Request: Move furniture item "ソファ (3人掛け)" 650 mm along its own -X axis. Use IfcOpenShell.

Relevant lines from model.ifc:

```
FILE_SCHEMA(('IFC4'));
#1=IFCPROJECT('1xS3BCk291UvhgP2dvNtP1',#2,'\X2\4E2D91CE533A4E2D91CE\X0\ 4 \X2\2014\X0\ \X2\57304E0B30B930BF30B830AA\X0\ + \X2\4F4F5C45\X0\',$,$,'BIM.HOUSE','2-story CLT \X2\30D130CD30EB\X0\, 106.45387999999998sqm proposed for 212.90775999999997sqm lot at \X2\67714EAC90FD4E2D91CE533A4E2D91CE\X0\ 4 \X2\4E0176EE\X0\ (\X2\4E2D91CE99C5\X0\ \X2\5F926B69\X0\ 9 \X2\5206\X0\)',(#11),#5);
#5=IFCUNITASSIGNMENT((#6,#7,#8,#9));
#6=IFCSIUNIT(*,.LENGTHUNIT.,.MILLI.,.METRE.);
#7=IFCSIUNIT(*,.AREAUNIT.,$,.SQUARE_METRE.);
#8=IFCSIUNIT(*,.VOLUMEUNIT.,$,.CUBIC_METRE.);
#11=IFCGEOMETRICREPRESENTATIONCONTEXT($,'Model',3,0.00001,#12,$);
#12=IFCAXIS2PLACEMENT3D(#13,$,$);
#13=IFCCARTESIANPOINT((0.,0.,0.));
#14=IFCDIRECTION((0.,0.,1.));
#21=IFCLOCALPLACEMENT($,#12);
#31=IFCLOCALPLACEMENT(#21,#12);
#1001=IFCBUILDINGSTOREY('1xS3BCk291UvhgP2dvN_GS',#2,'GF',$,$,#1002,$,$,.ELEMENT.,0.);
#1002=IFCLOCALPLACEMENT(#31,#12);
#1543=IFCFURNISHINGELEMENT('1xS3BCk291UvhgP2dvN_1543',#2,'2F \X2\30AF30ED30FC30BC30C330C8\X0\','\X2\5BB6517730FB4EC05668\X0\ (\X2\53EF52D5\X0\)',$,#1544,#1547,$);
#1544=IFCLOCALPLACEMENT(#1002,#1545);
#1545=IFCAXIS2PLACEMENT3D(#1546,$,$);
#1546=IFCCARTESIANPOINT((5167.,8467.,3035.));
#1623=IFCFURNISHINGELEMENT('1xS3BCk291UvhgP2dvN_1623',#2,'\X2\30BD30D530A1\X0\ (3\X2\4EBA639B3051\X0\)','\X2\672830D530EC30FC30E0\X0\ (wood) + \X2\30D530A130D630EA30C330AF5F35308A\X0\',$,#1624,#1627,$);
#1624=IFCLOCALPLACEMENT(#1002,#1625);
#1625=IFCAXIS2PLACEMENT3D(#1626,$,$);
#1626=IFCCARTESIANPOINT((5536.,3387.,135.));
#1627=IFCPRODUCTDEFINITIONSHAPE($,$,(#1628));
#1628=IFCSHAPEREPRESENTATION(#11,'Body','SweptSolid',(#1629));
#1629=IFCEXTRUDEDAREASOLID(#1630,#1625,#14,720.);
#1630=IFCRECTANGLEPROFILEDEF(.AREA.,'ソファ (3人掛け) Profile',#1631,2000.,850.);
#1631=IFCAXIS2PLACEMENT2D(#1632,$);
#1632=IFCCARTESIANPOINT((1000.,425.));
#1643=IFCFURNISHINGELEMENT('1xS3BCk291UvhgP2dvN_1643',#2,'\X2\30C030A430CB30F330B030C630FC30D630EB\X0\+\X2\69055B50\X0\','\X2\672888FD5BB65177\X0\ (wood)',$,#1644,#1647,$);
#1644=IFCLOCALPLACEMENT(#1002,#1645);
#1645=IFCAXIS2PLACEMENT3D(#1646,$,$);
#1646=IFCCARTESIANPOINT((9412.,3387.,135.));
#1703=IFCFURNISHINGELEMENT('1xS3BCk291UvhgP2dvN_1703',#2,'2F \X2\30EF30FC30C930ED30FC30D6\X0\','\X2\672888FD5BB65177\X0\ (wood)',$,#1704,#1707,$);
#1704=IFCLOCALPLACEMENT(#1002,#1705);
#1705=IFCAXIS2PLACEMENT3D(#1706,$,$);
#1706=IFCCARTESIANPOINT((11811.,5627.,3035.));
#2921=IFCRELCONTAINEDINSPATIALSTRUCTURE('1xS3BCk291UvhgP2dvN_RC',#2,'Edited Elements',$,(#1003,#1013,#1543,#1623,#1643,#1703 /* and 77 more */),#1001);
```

```python
import ifcopenshell
import ifcopenshell.api.geometry
import ifcopenshell.util.placement

model = ifcopenshell.open("model.ifc")

item = model.by_id(1623)
matrix = ifcopenshell.util.placement.get_local_placement(item.ObjectPlacement)
matrix[:3, 3] -= matrix[:3, 0] * 650.0
ifcopenshell.api.geometry.edit_object_placement(model, product=item, matrix=matrix, is_si=False)

print(ifcopenshell.util.placement.get_local_placement(item.ObjectPlacement).round(3) + 0.0)

model.write("model-out.ifc")
```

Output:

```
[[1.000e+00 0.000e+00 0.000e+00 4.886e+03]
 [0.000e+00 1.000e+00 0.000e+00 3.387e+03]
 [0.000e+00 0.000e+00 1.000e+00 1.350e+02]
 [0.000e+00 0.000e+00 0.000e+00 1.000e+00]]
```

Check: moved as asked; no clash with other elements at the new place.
